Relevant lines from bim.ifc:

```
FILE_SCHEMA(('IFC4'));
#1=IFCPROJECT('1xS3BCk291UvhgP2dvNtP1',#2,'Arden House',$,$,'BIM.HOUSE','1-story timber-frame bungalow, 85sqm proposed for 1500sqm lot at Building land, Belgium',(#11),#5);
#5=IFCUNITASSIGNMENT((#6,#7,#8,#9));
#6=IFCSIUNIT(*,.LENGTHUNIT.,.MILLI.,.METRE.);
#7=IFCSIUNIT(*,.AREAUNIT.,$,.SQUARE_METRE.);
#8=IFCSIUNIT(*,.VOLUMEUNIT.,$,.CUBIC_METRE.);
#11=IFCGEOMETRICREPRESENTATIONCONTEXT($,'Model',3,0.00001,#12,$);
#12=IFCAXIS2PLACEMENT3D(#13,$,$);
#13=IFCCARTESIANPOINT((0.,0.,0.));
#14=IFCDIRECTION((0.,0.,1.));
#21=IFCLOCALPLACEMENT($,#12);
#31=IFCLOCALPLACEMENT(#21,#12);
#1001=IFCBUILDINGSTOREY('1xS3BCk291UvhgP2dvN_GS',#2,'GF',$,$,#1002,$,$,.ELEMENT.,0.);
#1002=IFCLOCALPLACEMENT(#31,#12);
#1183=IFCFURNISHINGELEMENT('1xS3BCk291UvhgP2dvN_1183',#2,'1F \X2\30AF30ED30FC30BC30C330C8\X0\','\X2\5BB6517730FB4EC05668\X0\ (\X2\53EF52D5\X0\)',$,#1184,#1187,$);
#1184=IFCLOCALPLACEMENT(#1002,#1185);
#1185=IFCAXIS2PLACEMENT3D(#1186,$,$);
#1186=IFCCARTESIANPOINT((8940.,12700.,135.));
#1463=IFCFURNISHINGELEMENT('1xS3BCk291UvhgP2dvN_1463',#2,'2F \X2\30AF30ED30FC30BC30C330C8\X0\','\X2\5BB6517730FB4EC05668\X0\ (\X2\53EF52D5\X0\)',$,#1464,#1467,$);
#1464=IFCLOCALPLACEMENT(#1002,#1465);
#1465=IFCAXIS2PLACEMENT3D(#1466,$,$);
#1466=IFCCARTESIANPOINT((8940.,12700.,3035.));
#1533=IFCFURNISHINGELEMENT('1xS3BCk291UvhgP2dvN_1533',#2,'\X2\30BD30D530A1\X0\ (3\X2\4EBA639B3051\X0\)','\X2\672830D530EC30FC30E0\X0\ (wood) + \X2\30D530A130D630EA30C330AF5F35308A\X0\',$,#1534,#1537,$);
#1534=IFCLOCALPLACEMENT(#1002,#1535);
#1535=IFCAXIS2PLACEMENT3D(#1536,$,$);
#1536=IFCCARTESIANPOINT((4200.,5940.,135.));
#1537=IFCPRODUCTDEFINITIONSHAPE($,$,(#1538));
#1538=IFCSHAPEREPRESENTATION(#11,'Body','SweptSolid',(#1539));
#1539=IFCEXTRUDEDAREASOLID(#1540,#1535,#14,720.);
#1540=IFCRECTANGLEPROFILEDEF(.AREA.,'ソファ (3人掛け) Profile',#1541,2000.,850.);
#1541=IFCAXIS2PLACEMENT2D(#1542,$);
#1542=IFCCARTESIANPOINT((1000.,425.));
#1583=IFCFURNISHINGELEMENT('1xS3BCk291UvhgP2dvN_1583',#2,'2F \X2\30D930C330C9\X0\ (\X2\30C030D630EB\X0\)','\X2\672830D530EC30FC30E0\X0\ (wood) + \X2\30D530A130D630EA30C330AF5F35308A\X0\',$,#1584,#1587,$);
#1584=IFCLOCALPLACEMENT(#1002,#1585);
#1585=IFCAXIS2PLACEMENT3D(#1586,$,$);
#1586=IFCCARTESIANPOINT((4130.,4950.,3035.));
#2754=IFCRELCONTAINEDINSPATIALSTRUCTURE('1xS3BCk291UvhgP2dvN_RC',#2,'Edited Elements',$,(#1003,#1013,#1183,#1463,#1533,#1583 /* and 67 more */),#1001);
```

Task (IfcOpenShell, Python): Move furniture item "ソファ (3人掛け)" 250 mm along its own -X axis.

```python
import ifcopenshell
import ifcopenshell.api.geometry
import ifcopenshell.util.placement
import ifcopenshell.util.unit

model = ifcopenshell.open("bim.ifc")
unit_scale = ifcopenshell.util.unit.calculate_unit_scale(model)

item = model.by_guid("1xS3BCk291UvhgP2dvN_1533")
matrix = ifcopenshell.util.placement.get_local_placement(item.ObjectPlacement)
matrix[:3, 3] -= matrix[:3, 0] * 0.25 / unit_scale
ifcopenshell.api.geometry.edit_object_placement(model, product=item, matrix=matrix, is_si=False)

print(ifcopenshell.util.placement.get_local_placement(item.ObjectPlacement).round(3) + 0.0)

model.write("bim_updated.ifc")
```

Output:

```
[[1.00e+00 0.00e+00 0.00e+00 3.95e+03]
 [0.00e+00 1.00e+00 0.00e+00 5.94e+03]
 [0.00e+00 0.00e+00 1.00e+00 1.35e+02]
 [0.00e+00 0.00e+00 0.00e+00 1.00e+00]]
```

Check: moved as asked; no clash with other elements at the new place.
